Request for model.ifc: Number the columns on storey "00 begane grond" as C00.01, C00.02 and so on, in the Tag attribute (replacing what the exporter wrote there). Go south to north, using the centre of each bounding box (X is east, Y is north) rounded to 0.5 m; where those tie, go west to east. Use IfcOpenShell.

First a look at what the model holds.

```python
import ifcopenshell
import ifcopenshell.util.element
import ifcopenshell.util.placement

model = ifcopenshell.open("model.ifc")
print(model.schema)
storey = next(s for s in model.by_type("IfcBuildingStorey") if s.Name == "00 begane grond")
columns = [e for e in ifcopenshell.util.element.get_decomposition(storey) if e.is_a("IfcColumn")]
for e in sorted(columns, key=lambda e: e.id()):
    origin = ifcopenshell.util.placement.get_local_placement(e.ObjectPlacement)[:3, 3]
    print(e.id(), e.Tag, e.Name, origin.round(2) + 0.0, sep=" | ")
```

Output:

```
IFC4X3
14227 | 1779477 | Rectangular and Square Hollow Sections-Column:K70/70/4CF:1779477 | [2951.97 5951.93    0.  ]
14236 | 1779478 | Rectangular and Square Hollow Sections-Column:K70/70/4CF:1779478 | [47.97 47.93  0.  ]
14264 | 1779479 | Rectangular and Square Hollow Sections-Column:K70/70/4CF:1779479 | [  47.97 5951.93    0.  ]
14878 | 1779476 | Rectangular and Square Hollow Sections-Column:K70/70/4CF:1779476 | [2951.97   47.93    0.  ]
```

```python
import ifcopenshell
import ifcopenshell.geom
import ifcopenshell.util.element
import ifcopenshell.util.shape

model = ifcopenshell.open("model.ifc")
settings = ifcopenshell.geom.settings()
settings.set("use-world-coords", True)


def centre(element):
    shape = ifcopenshell.geom.create_shape(settings, element)
    return ifcopenshell.util.shape.get_bbox_centroid(shape.geometry)


storey = next(s for s in model.by_type("IfcBuildingStorey") if s.Name == "00 begane grond")
columns = [e for e in ifcopenshell.util.element.get_decomposition(storey) if e.is_a("IfcColumn")]

# Insertion points can sit at a corner or the storey origin, so sort by the geometry (in metres).
centres = {e: centre(e) for e in columns}
columns.sort(key=lambda e: (round(centres[e][1] / 0.5), centres[e][0]))

for i, e in enumerate(columns, start=1):
    number = f"C00.{i:02d}"
    e.Tag = number
    print(e.id(), number)

model.write("model_rev.ifc")
```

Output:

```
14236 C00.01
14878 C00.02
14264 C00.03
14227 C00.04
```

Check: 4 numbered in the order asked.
